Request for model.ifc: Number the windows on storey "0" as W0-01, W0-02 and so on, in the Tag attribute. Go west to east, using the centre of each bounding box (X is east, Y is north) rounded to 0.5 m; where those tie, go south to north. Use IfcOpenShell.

First a look at what the model holds.

```python
import ifcopenshell
import ifcopenshell.util.element
import ifcopenshell.util.placement

model = ifcopenshell.open("model.ifc")
print(model.schema)
storey = next(s for s in model.by_type("IfcBuildingStorey") if s.Name == "0")
windows = [e for e in ifcopenshell.util.element.get_decomposition(storey) if e.is_a("IfcWindow")]
for e in sorted(windows, key=lambda e: e.id()):
    origin = ifcopenshell.util.placement.get_local_placement(e.ObjectPlacement)[:3, 3]
    print(e.id(), e.Tag, e.Name, origin.round(2) + 0.0, sep=" | ")
```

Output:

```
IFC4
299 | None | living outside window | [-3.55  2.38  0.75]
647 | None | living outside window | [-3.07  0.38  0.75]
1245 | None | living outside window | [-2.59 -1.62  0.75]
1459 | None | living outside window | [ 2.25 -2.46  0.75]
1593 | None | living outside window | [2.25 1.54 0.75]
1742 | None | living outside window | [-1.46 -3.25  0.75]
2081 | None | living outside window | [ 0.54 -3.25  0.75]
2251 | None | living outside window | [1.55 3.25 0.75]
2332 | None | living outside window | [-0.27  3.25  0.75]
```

```python
import ifcopenshell
import ifcopenshell.geom
import ifcopenshell.util.element
import ifcopenshell.util.shape

model = ifcopenshell.open("model.ifc")
settings = ifcopenshell.geom.settings()
settings.set("use-world-coords", True)


def centre(element):
    shape = ifcopenshell.geom.create_shape(settings, element)
    return ifcopenshell.util.shape.get_bbox_centroid(shape.geometry)


storey = next(s for s in model.by_type("IfcBuildingStorey") if s.Name == "0")
windows = [e for e in ifcopenshell.util.element.get_decomposition(storey) if e.is_a("IfcWindow")]

# Insertion points can sit at a corner or the storey origin, so sort by the geometry (in metres).
centres = {e: centre(e) for e in windows}
windows.sort(key=lambda e: (round(centres[e][0] / 0.5), centres[e][1]))

for i, e in enumerate(windows, start=1):
    number = f"W0-{i:02d}"
    e.Tag = number
    print(e.id(), number)

model.write("model-out.ifc")
```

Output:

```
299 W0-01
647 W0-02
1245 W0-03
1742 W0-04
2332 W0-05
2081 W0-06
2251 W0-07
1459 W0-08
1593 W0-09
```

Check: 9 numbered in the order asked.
